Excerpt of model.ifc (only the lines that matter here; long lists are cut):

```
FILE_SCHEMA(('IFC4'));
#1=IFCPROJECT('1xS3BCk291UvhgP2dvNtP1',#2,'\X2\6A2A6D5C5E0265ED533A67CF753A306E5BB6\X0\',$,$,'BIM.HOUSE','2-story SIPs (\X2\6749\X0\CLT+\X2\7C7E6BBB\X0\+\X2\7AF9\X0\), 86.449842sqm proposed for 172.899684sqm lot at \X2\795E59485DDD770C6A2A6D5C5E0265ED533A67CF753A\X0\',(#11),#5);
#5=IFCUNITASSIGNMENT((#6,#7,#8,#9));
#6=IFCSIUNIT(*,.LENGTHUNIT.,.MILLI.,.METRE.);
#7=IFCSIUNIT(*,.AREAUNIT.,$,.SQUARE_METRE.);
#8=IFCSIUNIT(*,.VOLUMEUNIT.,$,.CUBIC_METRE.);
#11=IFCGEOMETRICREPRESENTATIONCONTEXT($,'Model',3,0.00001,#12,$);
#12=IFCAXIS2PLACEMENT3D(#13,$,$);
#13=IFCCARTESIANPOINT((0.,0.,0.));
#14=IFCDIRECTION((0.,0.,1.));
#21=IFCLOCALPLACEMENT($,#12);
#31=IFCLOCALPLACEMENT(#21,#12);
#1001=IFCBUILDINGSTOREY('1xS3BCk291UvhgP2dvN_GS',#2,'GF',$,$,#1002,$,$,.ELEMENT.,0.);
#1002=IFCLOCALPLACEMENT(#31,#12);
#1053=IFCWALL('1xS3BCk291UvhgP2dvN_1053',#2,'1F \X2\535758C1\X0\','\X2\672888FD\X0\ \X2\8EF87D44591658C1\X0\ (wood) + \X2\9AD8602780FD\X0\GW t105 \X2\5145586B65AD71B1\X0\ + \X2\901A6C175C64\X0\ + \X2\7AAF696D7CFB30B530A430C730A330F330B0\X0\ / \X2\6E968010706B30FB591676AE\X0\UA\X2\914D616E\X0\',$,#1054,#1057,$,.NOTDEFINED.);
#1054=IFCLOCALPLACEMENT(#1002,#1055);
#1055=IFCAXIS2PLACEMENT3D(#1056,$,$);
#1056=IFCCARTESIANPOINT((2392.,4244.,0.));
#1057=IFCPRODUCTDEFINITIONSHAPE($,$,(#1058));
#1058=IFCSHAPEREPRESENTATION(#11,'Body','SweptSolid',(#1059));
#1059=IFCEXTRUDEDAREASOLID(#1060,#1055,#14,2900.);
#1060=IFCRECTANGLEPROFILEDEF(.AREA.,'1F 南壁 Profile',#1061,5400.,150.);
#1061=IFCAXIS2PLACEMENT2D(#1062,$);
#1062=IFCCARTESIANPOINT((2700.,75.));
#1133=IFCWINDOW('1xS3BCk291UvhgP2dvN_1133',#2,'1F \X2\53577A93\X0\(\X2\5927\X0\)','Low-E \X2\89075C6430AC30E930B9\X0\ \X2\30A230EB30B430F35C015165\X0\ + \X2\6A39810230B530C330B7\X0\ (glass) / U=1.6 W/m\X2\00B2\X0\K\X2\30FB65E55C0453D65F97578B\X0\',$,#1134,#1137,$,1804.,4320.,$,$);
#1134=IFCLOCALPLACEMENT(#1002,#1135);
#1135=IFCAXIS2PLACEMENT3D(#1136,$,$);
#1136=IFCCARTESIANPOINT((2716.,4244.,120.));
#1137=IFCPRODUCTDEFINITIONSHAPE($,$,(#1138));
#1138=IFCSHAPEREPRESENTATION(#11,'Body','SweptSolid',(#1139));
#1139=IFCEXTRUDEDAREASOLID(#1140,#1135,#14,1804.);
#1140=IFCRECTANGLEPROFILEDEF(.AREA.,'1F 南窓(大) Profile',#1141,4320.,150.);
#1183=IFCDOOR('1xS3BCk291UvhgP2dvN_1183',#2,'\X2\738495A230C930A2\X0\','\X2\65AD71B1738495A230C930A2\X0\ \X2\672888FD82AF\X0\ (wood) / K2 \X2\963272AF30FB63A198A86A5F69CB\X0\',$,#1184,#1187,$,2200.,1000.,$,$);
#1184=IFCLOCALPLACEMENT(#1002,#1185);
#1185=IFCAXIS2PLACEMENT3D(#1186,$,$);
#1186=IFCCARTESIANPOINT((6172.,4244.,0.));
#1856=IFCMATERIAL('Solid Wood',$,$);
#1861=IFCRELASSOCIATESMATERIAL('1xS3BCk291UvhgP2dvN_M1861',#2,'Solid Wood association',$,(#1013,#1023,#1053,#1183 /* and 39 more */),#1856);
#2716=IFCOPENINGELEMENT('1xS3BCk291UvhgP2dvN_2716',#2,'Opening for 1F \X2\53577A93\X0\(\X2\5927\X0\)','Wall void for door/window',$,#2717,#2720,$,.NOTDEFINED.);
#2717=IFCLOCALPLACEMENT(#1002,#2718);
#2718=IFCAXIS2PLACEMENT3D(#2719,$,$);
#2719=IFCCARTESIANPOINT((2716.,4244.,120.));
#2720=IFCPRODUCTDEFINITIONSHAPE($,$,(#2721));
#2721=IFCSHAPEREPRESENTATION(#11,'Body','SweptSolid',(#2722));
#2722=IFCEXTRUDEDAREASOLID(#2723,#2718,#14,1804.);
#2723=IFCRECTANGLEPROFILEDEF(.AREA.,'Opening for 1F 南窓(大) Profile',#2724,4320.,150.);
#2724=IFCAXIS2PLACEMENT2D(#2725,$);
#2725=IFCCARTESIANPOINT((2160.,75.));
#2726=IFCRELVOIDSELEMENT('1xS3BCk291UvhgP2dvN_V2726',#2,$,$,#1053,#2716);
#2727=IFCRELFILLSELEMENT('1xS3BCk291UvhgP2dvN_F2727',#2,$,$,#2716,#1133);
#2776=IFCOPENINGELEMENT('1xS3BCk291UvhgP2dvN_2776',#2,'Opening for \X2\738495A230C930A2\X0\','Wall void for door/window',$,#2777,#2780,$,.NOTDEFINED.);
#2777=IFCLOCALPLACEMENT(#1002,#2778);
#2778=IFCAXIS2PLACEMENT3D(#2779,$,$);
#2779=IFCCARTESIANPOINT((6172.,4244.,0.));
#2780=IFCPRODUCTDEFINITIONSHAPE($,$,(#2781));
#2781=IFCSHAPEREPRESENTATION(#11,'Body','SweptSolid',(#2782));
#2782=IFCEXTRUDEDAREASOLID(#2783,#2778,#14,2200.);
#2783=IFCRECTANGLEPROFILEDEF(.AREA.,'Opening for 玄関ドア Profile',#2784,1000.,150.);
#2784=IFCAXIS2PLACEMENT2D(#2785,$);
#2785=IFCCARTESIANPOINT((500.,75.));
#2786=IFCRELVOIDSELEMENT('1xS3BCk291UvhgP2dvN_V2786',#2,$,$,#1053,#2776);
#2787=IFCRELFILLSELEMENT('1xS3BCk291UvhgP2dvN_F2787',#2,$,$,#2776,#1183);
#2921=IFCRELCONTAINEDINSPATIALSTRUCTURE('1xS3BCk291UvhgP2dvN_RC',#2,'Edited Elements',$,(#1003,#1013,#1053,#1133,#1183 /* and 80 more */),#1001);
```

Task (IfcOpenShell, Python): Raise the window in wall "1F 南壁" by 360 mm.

```python
import numpy as np
import ifcopenshell
import ifcopenshell.api.geometry
import ifcopenshell.util.placement
import ifcopenshell.util.unit

model = ifcopenshell.open("model.ifc")
unit_scale = ifcopenshell.util.unit.calculate_unit_scale(model)

window = model.by_id(1133)
opening = window.FillsVoids[0].RelatingOpeningElement
dz = 0.36 / unit_scale

shift = np.array([0.0, 0.0, dz])
# The window is not placed relative to its opening, so move both.
for product in (opening, window):
    matrix = ifcopenshell.util.placement.get_local_placement(product.ObjectPlacement)
    matrix[:3, 3] += shift
    ifcopenshell.api.geometry.edit_object_placement(model, product=product, matrix=matrix, is_si=False)

print(f"moved by {dz * unit_scale:+.3f} m")

model.write("model_rev.ifc")
```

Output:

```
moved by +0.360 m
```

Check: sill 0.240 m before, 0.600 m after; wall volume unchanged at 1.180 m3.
